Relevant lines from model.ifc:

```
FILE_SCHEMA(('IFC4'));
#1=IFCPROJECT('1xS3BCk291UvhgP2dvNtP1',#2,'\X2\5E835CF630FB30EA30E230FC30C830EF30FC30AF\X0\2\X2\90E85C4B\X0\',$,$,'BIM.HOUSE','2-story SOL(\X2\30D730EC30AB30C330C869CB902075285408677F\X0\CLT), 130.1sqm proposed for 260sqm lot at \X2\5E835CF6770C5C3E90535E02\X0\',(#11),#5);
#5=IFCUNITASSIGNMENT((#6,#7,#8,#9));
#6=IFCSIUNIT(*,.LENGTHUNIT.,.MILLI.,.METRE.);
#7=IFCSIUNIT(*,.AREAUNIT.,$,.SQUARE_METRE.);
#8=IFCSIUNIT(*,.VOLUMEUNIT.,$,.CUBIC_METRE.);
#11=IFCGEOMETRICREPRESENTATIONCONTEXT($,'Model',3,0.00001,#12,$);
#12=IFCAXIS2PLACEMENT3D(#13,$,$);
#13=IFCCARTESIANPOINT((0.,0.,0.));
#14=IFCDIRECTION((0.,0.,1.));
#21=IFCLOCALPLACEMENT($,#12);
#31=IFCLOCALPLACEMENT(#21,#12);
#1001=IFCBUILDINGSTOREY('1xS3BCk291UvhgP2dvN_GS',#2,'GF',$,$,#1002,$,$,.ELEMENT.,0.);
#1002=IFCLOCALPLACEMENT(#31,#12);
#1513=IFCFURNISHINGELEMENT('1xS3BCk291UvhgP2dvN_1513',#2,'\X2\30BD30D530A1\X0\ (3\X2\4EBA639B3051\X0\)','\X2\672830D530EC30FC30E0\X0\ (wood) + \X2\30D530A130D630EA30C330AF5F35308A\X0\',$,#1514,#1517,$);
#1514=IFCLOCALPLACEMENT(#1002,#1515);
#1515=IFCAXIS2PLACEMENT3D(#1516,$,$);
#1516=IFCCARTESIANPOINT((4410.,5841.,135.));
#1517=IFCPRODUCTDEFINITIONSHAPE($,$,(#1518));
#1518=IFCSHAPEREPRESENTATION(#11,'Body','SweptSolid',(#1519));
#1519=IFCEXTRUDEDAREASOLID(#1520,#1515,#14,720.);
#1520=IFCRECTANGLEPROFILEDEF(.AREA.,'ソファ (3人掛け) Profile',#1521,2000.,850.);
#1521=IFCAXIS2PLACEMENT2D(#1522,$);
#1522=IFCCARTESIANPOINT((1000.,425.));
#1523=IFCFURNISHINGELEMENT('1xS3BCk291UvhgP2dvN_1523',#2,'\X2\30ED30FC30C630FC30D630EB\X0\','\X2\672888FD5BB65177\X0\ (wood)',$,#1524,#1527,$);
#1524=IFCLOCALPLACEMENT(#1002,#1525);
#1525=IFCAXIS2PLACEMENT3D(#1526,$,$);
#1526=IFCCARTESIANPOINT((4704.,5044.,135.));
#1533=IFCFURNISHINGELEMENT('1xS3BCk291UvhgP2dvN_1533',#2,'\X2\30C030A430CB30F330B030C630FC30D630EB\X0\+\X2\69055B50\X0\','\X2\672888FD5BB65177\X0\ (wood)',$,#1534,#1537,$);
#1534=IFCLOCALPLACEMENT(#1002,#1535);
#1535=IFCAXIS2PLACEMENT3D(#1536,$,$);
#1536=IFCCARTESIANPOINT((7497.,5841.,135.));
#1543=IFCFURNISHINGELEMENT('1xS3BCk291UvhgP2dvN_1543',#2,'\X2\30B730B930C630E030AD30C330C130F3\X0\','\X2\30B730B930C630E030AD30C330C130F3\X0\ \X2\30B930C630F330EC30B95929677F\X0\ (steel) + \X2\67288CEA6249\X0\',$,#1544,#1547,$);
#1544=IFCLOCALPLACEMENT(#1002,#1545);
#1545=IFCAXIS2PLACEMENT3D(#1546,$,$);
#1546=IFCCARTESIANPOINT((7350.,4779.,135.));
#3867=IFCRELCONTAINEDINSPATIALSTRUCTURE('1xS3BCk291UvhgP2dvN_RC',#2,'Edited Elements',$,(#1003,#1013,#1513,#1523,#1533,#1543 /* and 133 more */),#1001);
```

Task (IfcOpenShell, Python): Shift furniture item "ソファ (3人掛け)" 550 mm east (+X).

```python
import ifcopenshell
import ifcopenshell.api.geometry
import ifcopenshell.util.placement

model = ifcopenshell.open("model.ifc")

item = model.by_guid("1xS3BCk291UvhgP2dvN_1513")
matrix = ifcopenshell.util.placement.get_local_placement(item.ObjectPlacement)
matrix[0, 3] += 550.0
ifcopenshell.api.geometry.edit_object_placement(model, product=item, matrix=matrix, is_si=False)

print(ifcopenshell.util.placement.get_local_placement(item.ObjectPlacement).round(3) + 0.0)

model.write("model_rev.ifc")
```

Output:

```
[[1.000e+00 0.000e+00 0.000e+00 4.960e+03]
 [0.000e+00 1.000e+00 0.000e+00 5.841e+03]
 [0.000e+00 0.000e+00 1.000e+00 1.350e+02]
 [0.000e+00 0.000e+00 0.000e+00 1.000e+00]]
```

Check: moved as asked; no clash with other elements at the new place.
